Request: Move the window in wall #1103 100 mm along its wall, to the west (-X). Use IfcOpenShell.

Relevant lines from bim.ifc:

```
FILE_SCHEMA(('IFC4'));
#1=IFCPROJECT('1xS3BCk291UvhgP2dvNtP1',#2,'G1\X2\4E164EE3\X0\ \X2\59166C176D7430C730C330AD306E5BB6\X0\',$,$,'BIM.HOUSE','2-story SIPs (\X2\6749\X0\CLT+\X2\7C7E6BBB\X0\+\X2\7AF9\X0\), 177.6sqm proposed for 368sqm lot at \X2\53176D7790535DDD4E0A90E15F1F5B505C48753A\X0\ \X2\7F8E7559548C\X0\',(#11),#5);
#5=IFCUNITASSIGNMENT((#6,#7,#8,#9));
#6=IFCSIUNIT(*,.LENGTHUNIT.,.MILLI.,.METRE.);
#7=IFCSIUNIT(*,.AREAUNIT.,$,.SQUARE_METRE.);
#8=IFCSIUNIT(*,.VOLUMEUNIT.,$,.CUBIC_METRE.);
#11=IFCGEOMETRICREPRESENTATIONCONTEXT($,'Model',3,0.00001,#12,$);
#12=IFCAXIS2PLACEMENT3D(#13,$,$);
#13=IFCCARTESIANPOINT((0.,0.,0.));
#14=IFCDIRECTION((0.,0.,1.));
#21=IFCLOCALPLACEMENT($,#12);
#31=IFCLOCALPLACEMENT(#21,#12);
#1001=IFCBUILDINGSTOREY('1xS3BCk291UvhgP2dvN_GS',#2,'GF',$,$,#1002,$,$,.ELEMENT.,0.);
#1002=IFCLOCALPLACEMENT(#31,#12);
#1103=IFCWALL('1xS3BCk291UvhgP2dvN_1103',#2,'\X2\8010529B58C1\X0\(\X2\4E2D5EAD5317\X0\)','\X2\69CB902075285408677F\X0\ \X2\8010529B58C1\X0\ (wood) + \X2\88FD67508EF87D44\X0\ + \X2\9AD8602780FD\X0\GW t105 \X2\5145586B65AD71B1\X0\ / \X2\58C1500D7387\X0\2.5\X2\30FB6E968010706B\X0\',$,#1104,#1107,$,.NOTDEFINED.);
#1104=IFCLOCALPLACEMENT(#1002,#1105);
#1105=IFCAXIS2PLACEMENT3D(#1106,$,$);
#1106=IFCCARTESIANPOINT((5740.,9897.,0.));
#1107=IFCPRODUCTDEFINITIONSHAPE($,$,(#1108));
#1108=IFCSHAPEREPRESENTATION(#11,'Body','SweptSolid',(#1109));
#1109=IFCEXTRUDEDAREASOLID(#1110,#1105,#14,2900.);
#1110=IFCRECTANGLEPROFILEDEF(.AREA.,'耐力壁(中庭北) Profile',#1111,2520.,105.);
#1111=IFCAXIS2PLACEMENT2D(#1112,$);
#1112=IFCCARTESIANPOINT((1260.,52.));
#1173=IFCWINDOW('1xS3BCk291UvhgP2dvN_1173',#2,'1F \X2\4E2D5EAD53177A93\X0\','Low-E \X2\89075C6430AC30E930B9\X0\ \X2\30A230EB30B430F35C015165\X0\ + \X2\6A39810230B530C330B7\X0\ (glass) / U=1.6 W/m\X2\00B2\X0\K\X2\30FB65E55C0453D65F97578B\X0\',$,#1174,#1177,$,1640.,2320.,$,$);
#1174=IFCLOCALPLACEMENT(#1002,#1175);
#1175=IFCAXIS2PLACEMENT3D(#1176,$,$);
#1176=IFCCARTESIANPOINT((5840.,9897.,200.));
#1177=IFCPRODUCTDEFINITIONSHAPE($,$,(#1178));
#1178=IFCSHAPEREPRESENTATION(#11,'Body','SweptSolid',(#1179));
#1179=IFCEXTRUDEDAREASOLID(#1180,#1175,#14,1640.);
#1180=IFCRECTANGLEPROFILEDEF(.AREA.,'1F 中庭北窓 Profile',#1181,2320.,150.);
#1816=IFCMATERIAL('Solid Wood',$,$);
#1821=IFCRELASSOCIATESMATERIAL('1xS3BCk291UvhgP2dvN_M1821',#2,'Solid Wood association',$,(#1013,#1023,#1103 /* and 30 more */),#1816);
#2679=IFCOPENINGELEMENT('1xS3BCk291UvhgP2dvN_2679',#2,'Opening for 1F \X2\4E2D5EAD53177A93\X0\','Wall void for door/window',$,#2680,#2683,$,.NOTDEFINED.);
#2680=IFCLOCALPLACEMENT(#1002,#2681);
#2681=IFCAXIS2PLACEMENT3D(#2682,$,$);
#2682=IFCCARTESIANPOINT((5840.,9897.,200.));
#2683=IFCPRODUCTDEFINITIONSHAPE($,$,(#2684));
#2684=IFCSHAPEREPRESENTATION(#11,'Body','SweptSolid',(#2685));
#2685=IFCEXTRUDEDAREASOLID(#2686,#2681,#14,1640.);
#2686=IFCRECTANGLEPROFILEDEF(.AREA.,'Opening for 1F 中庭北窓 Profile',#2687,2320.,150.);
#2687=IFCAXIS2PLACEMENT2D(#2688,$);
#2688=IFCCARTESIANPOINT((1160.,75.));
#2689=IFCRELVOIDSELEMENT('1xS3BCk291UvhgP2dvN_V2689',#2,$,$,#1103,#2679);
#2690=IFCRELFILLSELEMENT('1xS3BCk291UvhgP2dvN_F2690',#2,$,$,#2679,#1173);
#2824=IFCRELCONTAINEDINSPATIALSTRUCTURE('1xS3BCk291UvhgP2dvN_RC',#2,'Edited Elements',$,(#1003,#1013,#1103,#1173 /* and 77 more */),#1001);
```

```python
import ifcopenshell
import ifcopenshell.api.geometry
import ifcopenshell.util.placement

model = ifcopenshell.open("bim.ifc")

window = model.by_guid("1xS3BCk291UvhgP2dvN_1173")
opening = window.FillsVoids[0].RelatingOpeningElement
wall = opening.VoidsElements[0].RelatingBuildingElement

wall_matrix = ifcopenshell.util.placement.get_local_placement(wall.ObjectPlacement)
shift = wall_matrix[:3, 0] * -100.0
before = ifcopenshell.util.placement.get_local_placement(window.ObjectPlacement)[:3, 3].copy()

# The window is not placed relative to its opening, so move both.
for product in (opening, window):
    matrix = ifcopenshell.util.placement.get_local_placement(product.ObjectPlacement)
    matrix[:3, 3] += shift
    ifcopenshell.api.geometry.edit_object_placement(model, product=product, matrix=matrix, is_si=False)

after = ifcopenshell.util.placement.get_local_placement(window.ObjectPlacement)[:3, 3]
print("window moved by", (after - before).round(3) + 0.0)

model.write("bim_rev.ifc")
```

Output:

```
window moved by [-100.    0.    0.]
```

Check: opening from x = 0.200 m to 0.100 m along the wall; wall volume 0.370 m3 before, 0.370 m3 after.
